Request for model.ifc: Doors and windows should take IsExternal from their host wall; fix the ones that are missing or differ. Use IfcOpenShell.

First a look at what the model holds.

```python
import ifcopenshell
import ifcopenshell.util.element

model = ifcopenshell.open("model.ifc")
print(model.schema)
seen = {}
for e in model.by_type("IfcDoor") + model.by_type("IfcWindow"):
    if not e.FillsVoids:
        continue
    host = e.FillsVoids[0].RelatingOpeningElement.VoidsElements[0].RelatingBuildingElement
    own = ifcopenshell.util.element.get_pset(e, f"Pset_{e.is_a()[3:].removesuffix('StandardCase')}Common", "IsExternal")
    wall = ifcopenshell.util.element.get_pset(host, "Pset_WallCommon", "IsExternal")
    seen[e.is_a(), own, wall] = seen.get((e.is_a(), own, wall), 0) + 1
for (cls, own, wall), count in sorted(seen.items(), key=str):
    print(count, cls, "IsExternal:", own, "| host wall:", wall)
```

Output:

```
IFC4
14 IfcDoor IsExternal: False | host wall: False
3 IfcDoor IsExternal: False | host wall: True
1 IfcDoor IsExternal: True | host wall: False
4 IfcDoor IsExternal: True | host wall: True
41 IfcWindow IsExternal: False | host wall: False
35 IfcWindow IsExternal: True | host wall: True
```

```python
import ifcopenshell
import ifcopenshell.api.pset
import ifcopenshell.util.element

model = ifcopenshell.open("model.ifc")

count = 0
for ifc_class, pset_name in (("IfcDoor", "Pset_DoorCommon"), ("IfcWindow", "Pset_WindowCommon")):
    for e in model.by_type(ifc_class):
        if not e.FillsVoids:
            continue
        host = e.FillsVoids[0].RelatingOpeningElement.VoidsElements[0].RelatingBuildingElement
        external = ifcopenshell.util.element.get_pset(host, "Pset_WallCommon", "IsExternal")
        if external is None or ifcopenshell.util.element.get_pset(e, pset_name, "IsExternal") == external:
            continue
        pset = ifcopenshell.api.pset.add_pset(model, product=e, name=pset_name)
        ifcopenshell.api.pset.edit_pset(model, pset=pset, properties={"IsExternal": external})
        count += 1

print(count, "updated")

model.write("model_v2.ifc")
```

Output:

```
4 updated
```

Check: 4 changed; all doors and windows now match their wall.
